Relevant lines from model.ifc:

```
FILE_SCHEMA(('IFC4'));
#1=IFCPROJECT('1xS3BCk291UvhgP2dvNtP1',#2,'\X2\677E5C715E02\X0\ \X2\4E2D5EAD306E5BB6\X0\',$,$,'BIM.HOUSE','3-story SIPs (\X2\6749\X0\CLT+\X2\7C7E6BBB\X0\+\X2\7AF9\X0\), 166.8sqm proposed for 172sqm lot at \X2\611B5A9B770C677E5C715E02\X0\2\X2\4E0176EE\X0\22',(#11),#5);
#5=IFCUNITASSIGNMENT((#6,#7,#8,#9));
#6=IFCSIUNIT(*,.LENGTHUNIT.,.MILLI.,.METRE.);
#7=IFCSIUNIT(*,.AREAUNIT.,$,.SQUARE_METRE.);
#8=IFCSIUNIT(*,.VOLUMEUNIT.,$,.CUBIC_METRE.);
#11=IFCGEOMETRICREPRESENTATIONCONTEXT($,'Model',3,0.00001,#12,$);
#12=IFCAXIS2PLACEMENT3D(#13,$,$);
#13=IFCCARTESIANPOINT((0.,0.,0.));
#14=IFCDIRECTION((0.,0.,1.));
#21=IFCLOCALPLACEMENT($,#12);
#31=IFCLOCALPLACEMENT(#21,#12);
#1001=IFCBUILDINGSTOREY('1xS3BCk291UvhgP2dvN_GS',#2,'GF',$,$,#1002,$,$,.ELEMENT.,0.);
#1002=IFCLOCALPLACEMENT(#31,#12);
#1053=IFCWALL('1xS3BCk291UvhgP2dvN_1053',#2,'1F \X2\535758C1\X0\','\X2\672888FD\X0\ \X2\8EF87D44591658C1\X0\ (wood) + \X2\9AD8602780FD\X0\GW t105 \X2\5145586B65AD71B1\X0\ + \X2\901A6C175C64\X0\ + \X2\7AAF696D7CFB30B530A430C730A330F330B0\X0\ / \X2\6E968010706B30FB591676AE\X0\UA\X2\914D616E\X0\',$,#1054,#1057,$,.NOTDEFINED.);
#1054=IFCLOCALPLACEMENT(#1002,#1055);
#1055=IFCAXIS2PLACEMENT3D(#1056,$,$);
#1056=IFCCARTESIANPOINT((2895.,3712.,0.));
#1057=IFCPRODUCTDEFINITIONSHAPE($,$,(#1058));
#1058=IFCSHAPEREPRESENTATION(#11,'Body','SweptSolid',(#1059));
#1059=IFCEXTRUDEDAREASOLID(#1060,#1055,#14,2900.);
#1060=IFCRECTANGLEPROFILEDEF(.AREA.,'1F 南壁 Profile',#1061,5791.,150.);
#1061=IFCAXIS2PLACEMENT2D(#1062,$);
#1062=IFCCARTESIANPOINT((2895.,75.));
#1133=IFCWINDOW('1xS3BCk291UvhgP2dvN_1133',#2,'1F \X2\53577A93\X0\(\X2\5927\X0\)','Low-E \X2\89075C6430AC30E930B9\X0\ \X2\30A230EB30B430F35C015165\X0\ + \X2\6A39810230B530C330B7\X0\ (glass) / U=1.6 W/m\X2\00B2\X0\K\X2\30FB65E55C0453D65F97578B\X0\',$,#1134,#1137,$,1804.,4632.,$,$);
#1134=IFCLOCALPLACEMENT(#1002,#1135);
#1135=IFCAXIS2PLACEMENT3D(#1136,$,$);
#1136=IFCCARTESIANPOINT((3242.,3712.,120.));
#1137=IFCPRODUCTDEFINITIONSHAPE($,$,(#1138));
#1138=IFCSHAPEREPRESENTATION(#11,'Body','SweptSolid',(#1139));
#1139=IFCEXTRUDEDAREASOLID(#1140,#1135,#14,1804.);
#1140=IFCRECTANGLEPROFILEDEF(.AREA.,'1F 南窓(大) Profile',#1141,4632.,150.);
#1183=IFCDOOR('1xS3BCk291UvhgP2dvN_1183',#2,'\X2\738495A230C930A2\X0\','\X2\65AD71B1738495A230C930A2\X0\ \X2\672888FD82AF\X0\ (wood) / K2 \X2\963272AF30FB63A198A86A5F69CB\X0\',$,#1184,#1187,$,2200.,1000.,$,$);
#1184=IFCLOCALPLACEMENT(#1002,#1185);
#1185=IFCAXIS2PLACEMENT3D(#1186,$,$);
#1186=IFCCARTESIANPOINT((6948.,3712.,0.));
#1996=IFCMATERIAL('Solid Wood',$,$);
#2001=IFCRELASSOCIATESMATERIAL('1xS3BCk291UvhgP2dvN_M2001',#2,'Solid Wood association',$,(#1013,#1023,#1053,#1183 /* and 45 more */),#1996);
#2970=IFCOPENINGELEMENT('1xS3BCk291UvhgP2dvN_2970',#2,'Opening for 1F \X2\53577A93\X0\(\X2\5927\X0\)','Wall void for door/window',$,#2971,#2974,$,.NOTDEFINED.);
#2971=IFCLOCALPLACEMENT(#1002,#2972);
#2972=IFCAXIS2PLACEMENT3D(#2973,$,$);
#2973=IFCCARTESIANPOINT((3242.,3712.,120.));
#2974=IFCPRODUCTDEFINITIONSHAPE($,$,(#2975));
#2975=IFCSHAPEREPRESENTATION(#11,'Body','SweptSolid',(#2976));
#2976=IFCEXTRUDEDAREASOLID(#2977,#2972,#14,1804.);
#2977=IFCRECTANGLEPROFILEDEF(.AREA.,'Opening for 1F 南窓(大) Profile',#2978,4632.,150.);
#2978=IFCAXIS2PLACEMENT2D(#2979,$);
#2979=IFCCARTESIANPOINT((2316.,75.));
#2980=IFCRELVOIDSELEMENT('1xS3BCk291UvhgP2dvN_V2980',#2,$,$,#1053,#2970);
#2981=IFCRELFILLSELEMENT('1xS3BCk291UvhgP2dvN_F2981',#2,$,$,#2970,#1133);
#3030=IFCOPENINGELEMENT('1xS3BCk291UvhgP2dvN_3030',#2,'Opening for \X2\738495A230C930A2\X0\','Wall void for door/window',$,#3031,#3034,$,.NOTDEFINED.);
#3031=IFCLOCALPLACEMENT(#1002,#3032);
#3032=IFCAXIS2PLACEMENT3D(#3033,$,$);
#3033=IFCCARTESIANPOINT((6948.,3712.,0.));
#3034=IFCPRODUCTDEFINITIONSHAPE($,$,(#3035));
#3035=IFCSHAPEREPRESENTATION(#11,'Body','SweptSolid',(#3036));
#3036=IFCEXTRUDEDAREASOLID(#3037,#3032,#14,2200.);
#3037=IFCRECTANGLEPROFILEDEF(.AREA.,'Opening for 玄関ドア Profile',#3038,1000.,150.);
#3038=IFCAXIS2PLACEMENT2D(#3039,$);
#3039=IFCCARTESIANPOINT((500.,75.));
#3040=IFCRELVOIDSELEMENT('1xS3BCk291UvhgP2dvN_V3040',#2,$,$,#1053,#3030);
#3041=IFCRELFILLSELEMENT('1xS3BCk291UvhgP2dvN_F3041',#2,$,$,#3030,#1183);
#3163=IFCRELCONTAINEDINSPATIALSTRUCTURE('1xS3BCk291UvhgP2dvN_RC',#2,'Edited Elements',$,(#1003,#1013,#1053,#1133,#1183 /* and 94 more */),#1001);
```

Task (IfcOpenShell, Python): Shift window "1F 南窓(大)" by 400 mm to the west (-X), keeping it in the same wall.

```python
import ifcopenshell
import ifcopenshell.api.geometry
import ifcopenshell.util.placement

model = ifcopenshell.open("model.ifc")

window = model.by_guid("1xS3BCk291UvhgP2dvN_1133")
opening = window.FillsVoids[0].RelatingOpeningElement
wall = opening.VoidsElements[0].RelatingBuildingElement

wall_matrix = ifcopenshell.util.placement.get_local_placement(wall.ObjectPlacement)
shift = wall_matrix[:3, 0] * -400.0
before = ifcopenshell.util.placement.get_local_placement(window.ObjectPlacement)[:3, 3].copy()

# The window is not placed relative to its opening, so move both.
for product in (opening, window):
    matrix = ifcopenshell.util.placement.get_local_placement(product.ObjectPlacement)
    matrix[:3, 3] += shift
    ifcopenshell.api.geometry.edit_object_placement(model, product=product, matrix=matrix, is_si=False)

after = ifcopenshell.util.placement.get_local_placement(window.ObjectPlacement)[:3, 3]
print("window moved by", (after - before).round(3) + 0.0)

model.write("model-out.ifc")
```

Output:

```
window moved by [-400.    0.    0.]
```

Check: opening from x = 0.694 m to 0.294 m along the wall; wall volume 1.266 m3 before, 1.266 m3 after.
